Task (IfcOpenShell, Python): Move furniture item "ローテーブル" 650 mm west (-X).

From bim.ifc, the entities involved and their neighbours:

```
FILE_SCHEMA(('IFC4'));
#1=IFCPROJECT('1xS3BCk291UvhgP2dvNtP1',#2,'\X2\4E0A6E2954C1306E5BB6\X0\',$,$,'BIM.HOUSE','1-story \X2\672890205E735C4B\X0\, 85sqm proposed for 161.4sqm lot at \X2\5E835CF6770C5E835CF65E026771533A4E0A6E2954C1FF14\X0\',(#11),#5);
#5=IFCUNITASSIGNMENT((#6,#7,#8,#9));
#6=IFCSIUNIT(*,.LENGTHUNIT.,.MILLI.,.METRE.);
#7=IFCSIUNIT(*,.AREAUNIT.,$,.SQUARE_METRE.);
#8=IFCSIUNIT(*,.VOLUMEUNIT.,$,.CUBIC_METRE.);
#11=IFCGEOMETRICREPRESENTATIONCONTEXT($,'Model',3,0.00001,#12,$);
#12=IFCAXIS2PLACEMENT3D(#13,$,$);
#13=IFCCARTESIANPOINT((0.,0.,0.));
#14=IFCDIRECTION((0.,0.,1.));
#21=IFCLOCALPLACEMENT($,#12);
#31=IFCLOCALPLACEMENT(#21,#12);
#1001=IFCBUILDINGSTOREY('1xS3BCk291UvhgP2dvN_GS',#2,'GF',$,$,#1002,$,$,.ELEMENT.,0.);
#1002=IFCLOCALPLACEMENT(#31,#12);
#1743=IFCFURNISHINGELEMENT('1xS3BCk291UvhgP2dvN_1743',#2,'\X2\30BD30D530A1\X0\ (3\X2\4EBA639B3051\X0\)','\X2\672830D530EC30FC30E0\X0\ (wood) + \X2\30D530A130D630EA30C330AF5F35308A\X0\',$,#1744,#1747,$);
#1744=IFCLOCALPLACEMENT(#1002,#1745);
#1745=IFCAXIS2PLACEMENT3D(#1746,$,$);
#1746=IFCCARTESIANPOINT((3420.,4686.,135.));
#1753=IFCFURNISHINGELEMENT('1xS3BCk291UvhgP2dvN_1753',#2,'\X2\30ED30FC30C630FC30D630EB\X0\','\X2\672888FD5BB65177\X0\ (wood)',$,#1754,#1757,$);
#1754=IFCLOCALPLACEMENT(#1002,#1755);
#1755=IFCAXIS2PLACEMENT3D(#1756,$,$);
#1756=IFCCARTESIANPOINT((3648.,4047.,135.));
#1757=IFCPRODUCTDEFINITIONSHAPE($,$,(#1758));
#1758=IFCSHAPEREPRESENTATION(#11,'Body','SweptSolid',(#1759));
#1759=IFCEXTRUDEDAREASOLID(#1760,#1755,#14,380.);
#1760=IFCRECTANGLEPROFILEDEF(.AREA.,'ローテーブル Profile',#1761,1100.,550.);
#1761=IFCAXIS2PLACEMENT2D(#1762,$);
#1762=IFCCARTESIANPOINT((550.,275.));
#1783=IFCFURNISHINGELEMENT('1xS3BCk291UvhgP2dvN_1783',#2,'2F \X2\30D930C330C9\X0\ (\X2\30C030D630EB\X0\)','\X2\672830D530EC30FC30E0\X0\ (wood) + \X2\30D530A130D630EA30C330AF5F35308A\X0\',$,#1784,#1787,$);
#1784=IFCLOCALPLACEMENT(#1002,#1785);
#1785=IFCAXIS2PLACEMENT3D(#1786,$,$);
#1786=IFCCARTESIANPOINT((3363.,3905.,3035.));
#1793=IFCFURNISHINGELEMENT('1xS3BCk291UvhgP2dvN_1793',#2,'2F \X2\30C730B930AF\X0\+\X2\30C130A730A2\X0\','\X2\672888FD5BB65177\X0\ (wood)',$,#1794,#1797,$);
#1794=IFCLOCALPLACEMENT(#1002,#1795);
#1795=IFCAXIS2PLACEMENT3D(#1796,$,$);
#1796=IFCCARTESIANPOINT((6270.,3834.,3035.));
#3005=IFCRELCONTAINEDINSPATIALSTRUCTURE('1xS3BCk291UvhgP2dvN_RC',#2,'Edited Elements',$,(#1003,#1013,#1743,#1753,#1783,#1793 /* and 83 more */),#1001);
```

```python
import ifcopenshell
import ifcopenshell.api.geometry
import ifcopenshell.util.placement

model = ifcopenshell.open("bim.ifc")

item = model.by_guid("1xS3BCk291UvhgP2dvN_1753")
matrix = ifcopenshell.util.placement.get_local_placement(item.ObjectPlacement)
matrix[0, 3] -= 650.0
ifcopenshell.api.geometry.edit_object_placement(model, product=item, matrix=matrix, is_si=False)

print(ifcopenshell.util.placement.get_local_placement(item.ObjectPlacement).round(3) + 0.0)

model.write("bim_v2.ifc")
```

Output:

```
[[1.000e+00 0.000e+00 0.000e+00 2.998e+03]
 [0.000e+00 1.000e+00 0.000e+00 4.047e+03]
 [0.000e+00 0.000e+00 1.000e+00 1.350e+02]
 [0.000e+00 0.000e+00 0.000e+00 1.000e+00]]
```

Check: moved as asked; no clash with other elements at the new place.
